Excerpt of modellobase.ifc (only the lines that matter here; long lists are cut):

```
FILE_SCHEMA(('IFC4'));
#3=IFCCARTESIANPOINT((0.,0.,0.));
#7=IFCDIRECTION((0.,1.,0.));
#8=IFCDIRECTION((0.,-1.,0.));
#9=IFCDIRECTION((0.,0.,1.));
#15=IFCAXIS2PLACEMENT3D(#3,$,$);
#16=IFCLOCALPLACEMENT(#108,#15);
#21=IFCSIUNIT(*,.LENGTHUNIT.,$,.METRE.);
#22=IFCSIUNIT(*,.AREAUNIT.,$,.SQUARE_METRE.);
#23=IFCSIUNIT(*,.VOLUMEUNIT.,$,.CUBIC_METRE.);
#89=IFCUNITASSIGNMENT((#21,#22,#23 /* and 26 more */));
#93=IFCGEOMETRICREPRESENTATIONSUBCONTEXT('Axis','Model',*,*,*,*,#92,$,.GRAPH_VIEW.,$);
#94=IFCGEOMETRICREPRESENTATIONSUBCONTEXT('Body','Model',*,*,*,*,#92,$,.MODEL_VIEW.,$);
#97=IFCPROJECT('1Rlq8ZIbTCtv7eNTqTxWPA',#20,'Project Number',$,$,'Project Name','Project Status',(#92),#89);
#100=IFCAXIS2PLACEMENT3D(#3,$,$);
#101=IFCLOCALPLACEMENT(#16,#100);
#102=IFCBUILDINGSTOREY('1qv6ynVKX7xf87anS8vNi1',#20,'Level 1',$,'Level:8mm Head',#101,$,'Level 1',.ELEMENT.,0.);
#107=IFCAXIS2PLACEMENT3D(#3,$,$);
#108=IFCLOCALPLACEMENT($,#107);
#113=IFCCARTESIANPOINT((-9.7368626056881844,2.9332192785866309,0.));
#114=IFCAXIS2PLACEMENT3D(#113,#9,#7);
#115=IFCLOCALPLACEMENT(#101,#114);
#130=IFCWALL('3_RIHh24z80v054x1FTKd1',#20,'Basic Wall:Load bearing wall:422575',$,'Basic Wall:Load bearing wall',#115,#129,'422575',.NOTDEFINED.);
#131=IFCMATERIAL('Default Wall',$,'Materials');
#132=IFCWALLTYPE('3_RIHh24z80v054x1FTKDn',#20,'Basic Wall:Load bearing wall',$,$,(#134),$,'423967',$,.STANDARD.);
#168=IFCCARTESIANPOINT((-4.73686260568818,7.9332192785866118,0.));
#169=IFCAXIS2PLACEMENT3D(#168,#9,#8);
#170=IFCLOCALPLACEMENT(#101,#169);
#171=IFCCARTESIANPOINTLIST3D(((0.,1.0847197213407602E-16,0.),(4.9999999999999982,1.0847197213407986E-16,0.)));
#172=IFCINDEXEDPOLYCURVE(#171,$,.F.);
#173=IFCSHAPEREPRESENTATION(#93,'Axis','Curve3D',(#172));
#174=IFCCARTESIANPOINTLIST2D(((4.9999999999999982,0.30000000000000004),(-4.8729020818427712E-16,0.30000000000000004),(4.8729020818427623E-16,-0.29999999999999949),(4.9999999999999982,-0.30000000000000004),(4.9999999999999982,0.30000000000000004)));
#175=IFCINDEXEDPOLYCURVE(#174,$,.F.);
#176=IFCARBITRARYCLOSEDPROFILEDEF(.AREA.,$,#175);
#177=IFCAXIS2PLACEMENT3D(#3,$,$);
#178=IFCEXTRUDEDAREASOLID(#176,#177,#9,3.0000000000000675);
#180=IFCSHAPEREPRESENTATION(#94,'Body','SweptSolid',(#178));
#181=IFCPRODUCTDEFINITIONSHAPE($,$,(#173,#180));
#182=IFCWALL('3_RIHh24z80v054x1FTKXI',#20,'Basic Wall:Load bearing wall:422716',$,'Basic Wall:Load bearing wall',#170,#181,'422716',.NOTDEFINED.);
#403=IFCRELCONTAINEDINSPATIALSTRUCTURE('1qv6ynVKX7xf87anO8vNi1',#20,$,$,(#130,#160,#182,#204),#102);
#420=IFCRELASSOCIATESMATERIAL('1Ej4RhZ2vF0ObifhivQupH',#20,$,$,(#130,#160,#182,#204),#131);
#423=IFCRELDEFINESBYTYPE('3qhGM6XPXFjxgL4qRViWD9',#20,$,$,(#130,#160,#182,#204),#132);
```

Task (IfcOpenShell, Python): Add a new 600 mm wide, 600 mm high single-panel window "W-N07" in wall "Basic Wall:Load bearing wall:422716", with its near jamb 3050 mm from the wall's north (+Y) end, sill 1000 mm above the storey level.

```python
import numpy as np
import ifcopenshell
import ifcopenshell.api.feature
import ifcopenshell.api.geometry
import ifcopenshell.api.root
import ifcopenshell.api.spatial
import ifcopenshell.geom
import ifcopenshell.util.element
import ifcopenshell.util.placement
import ifcopenshell.util.representation
import ifcopenshell.util.shape
import ifcopenshell.util.unit

model = ifcopenshell.open("modellobase.ifc")
unit_scale = ifcopenshell.util.unit.calculate_unit_scale(model)
settings = ifcopenshell.geom.settings()


def volume(element):
    """Net volume in cubic metres, openings subtracted."""
    shape = ifcopenshell.geom.create_shape(settings, element)
    return ifcopenshell.util.shape.get_volume(shape.geometry)


wall = model.by_guid("3_RIHh24z80v054x1FTKXI")
storey = ifcopenshell.util.element.get_container(wall, ifc_class="IfcBuildingStorey")
context = ifcopenshell.util.representation.get_context(model, "Model", "Body", "MODEL_VIEW")
before = volume(wall)

width, height, from_end, sill = 0.6, 0.6, 3.05, 1  # metres

# The wall runs along its own X axis, and the end named is its -X end.
wall_shape = ifcopenshell.geom.create_shape(settings, wall)
x, y, z = ifcopenshell.util.shape.get_vertices(wall_shape.geometry).T
start = x.min() + from_end
face, thickness = float(y.min()), float(y.max() - y.min())
wall_matrix = ifcopenshell.util.placement.get_local_placement(wall.ObjectPlacement)
level = ifcopenshell.util.placement.get_local_placement(storey.ObjectPlacement)[2, 3]


def in_wall(x, y):
    """Placement at x, y metres in the wall's axes, at sill height."""
    matrix = wall_matrix.copy()
    matrix[:, 3] = wall_matrix @ np.array([x / unit_scale, y / unit_scale, 0.0, 1.0])
    matrix[2, 3] = level + sill / unit_scale
    return matrix


# Opening: a box that overshoots both wall faces by 50 mm.
opening = ifcopenshell.api.root.create_entity(model, ifc_class="IfcOpeningElement", predefined_type="OPENING")
box = ifcopenshell.api.geometry.add_wall_representation(
    model, context=context, length=width, height=height, thickness=thickness + 0.1
)
ifcopenshell.api.geometry.assign_representation(model, product=opening, representation=box)
ifcopenshell.api.geometry.edit_object_placement(model, product=opening, matrix=in_wall(start, face - 0.05), is_si=False)
ifcopenshell.api.feature.add_feature(model, feature=opening, element=wall)

window = ifcopenshell.api.root.create_entity(model, ifc_class="IfcWindow", name="W-N07", predefined_type="WINDOW")
window.OverallWidth, window.OverallHeight = width / unit_scale, height / unit_scale
window.PartitioningType = "SINGLE_PANEL"
body = ifcopenshell.api.geometry.add_window_representation(
    model,
    context=context,
    overall_width=window.OverallWidth,
    overall_height=window.OverallHeight,
    partition_type="SINGLE_PANEL",
)
ifcopenshell.api.geometry.assign_representation(model, product=window, representation=body)
ifcopenshell.api.spatial.assign_container(model, products=[window], relating_structure=storey)
ifcopenshell.api.feature.add_filling(model, opening=opening, element=window)

# Centre the window in the wall's thickness.
ifcopenshell.api.geometry.edit_object_placement(model, product=window, matrix=in_wall(start, face), is_si=False)
window_shape = ifcopenshell.geom.create_shape(settings, window)
depth = ifcopenshell.util.shape.get_vertices(window_shape.geometry)[:, 1]
offset = face + thickness / 2 - (depth.min() + depth.max()) / 2
ifcopenshell.api.geometry.edit_object_placement(model, product=window, matrix=in_wall(start, offset), is_si=False)

after = volume(wall)

print(f"wall volume {before:.3f} -> {after:.3f} m3")

model.write("modellobase_edited.ifc")
```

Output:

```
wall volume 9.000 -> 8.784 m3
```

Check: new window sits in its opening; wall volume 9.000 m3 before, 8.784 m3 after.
